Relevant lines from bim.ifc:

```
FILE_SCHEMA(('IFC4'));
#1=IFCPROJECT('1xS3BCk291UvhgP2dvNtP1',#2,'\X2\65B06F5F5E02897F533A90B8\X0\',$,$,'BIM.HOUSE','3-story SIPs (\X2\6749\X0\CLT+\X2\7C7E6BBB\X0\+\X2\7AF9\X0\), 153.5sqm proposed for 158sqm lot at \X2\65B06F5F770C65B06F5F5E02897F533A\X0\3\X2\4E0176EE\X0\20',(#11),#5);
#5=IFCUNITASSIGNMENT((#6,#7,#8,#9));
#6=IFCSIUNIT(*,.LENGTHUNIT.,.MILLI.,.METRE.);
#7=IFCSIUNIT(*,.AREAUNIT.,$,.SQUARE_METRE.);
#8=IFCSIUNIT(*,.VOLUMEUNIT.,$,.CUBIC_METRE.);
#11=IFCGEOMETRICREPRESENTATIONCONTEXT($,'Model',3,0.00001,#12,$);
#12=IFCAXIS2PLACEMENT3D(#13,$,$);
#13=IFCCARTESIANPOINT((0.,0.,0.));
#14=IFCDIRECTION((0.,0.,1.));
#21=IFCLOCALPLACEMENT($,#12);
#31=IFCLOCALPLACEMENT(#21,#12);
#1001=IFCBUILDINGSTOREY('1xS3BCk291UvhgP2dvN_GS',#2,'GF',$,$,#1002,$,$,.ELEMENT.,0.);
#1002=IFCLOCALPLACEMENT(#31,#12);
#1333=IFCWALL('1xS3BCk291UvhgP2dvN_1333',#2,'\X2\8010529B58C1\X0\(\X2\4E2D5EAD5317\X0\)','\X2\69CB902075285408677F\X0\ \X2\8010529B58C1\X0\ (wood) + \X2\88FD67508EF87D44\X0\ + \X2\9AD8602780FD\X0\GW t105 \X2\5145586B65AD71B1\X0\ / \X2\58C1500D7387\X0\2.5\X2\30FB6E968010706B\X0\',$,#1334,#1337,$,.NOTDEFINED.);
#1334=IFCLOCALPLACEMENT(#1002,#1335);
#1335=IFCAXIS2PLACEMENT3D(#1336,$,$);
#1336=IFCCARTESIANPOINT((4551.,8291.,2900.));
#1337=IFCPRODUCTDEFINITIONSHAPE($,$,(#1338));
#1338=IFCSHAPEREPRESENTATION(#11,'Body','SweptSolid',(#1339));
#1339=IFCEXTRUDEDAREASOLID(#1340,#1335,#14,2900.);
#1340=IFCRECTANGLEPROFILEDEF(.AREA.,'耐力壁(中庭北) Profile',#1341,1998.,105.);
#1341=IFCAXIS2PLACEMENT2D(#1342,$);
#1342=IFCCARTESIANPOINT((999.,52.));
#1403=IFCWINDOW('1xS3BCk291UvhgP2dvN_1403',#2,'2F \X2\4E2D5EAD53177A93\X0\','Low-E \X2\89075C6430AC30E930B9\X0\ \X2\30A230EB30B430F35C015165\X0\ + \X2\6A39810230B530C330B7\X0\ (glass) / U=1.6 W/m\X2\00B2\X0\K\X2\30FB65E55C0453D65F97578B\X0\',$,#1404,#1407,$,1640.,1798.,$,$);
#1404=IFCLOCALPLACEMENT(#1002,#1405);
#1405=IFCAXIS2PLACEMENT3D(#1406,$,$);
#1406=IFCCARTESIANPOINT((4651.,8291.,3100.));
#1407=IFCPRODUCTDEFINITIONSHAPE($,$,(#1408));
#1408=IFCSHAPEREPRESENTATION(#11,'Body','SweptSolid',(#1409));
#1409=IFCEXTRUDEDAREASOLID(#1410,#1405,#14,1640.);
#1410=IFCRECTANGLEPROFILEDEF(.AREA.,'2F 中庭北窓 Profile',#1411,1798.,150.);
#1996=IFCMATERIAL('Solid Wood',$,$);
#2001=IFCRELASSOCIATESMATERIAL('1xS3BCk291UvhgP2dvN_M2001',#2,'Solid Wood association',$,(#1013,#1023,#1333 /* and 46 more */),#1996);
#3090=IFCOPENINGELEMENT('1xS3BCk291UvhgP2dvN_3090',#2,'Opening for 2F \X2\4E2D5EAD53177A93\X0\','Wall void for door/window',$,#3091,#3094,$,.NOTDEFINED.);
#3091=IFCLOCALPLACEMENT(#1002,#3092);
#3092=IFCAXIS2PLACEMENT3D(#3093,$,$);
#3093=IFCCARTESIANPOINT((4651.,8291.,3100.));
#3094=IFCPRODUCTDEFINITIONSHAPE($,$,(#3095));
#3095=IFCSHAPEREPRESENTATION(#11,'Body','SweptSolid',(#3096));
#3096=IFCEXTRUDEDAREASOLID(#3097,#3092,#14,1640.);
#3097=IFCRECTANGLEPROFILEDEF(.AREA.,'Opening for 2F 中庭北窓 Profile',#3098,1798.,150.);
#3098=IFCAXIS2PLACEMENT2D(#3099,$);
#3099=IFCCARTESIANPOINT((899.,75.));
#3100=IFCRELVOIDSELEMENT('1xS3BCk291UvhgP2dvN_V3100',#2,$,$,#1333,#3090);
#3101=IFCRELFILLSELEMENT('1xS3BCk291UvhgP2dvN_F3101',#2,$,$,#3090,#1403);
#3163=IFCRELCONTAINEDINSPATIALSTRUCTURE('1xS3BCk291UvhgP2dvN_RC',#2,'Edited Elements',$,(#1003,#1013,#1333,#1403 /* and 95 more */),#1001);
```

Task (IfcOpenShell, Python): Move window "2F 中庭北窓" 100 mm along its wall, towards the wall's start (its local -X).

```python
import ifcopenshell
import ifcopenshell.api.geometry
import ifcopenshell.util.placement
import ifcopenshell.util.unit

model = ifcopenshell.open("bim.ifc")
unit_scale = ifcopenshell.util.unit.calculate_unit_scale(model)

window = model.by_id(1403)
opening = window.FillsVoids[0].RelatingOpeningElement
wall = opening.VoidsElements[0].RelatingBuildingElement

wall_matrix = ifcopenshell.util.placement.get_local_placement(wall.ObjectPlacement)
shift = wall_matrix[:3, 0] * -0.1 / unit_scale
before = ifcopenshell.util.placement.get_local_placement(window.ObjectPlacement)[:3, 3].copy()

# The window is not placed relative to its opening, so move both.
for product in (opening, window):
    matrix = ifcopenshell.util.placement.get_local_placement(product.ObjectPlacement)
    matrix[:3, 3] += shift
    ifcopenshell.api.geometry.edit_object_placement(model, product=product, matrix=matrix, is_si=False)

after = ifcopenshell.util.placement.get_local_placement(window.ObjectPlacement)[:3, 3]
print("window moved by", (after - before).round(3) + 0.0)

model.write("bim_updated.ifc")
```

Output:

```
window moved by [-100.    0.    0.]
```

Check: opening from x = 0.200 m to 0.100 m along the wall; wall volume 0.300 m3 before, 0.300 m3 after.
